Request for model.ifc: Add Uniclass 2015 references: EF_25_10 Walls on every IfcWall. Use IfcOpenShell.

First a look at what the model holds.

```python
import ifcopenshell

model = ifcopenshell.open("model.ifc")
print(model.schema)
print("classifications:", [c.Name for c in model.by_type("IfcClassification")])
for ifc_class in ("IfcDoor", "IfcRoof", "IfcStair", "IfcWall", "IfcWindow"):
    print(ifc_class, len(model.by_type(ifc_class)))
```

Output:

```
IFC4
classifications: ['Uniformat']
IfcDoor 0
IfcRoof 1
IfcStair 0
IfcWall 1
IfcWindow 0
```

```python
import ifcopenshell
import ifcopenshell.api.classification

model = ifcopenshell.open("model.ifc")

system = ifcopenshell.api.classification.add_classification(model, classification="Uniclass 2015")

codes = {
    "IfcWall": ("EF_25_10", "Walls"),
}
for ifc_class, (code, name) in codes.items():
    products = model.by_type(ifc_class)
    ifcopenshell.api.classification.add_reference(
        model, products=products, classification=system, identification=code, name=name
    )
    print(code, len(products))

model.write("model_rev.ifc")
```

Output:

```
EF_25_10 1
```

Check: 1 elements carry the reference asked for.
